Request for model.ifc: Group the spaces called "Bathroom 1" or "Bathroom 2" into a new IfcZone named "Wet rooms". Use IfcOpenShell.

First a look at what the model holds.

```python
import ifcopenshell

model = ifcopenshell.open("model.ifc")
print(model.schema)
seen = {}
for space in model.by_type("IfcSpace"):
    seen[space.LongName] = seen.get(space.LongName, 0) + 1
for name, count in sorted(seen.items(), key=str):
    print(count, "x", name)
print("zones:", [z.Name for z in model.by_type("IfcZone")][:20])
```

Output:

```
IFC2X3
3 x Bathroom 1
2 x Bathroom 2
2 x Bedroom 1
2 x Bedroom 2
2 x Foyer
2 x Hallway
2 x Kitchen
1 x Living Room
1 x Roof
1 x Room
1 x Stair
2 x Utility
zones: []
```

```python
import ifcopenshell
import ifcopenshell.api.group
import ifcopenshell.api.root

model = ifcopenshell.open("model.ifc")

names = {"Bathroom 1", "Bathroom 2"}
spaces = [s for s in model.by_type("IfcSpace") if s.LongName in names]

zone = ifcopenshell.api.root.create_entity(model, ifc_class="IfcZone", name="Wet rooms")
ifcopenshell.api.group.assign_group(model, products=spaces, group=zone)
print(len(spaces), "spaces in", zone.Name)

model.write("model_edited.ifc")
```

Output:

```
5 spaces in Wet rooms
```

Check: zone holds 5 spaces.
